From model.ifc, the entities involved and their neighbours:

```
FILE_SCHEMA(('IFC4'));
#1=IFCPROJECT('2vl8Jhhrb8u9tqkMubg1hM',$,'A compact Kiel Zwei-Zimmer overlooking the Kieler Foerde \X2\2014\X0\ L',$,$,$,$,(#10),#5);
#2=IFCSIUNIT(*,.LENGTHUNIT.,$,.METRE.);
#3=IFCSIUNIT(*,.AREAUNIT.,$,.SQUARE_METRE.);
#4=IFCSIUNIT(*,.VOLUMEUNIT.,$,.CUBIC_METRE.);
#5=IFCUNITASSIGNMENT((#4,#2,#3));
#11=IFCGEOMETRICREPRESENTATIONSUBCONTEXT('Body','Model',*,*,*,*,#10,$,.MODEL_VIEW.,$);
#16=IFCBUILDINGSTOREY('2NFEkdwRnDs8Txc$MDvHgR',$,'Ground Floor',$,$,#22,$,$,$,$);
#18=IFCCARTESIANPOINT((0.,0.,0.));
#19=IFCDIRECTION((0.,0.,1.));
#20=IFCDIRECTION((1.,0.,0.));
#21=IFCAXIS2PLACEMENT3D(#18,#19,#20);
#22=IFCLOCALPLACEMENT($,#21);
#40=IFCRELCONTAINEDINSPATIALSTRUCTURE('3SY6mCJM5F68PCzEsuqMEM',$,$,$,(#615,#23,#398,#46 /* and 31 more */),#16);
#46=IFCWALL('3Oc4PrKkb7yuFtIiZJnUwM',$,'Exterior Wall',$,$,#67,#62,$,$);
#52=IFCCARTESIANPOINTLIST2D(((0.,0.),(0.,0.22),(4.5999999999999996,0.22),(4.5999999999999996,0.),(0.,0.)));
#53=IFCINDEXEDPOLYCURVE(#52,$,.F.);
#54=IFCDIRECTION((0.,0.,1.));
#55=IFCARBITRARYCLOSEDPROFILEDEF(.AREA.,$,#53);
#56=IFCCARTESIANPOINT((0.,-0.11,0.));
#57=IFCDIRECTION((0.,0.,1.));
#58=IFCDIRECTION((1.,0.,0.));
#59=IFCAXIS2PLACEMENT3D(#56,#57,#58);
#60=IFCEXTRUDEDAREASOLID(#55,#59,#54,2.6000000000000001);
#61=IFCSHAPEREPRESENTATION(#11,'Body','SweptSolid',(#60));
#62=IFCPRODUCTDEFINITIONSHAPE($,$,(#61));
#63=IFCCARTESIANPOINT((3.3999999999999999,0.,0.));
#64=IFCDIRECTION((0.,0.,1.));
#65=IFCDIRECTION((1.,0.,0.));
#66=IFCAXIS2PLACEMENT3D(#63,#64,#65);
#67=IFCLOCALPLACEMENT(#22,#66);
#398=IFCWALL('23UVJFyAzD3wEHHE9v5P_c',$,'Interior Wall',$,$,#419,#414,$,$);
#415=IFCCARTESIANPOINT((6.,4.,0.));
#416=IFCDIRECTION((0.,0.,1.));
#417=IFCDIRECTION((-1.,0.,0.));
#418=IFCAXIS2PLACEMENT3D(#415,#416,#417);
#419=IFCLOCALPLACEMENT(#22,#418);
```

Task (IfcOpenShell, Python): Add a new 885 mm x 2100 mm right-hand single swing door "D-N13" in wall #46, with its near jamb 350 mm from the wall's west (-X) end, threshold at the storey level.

```python
import numpy as np
import ifcopenshell
import ifcopenshell.api.feature
import ifcopenshell.api.geometry
import ifcopenshell.api.root
import ifcopenshell.api.spatial
import ifcopenshell.geom
import ifcopenshell.util.element
import ifcopenshell.util.placement
import ifcopenshell.util.representation
import ifcopenshell.util.shape
import ifcopenshell.util.unit

model = ifcopenshell.open("model.ifc")
unit_scale = ifcopenshell.util.unit.calculate_unit_scale(model)
settings = ifcopenshell.geom.settings()


def volume(element):
    """Net volume in cubic metres, openings subtracted."""
    shape = ifcopenshell.geom.create_shape(settings, element)
    return ifcopenshell.util.shape.get_volume(shape.geometry)


wall = model.by_guid("3Oc4PrKkb7yuFtIiZJnUwM")
storey = ifcopenshell.util.element.get_container(wall, ifc_class="IfcBuildingStorey")
context = ifcopenshell.util.representation.get_context(model, "Model", "Body", "MODEL_VIEW")
before = volume(wall)

width, height, from_end, sill = 0.885, 2.1, 0.35, 0.0  # metres

# The wall runs along its own X axis, and the end named is its -X end.
wall_shape = ifcopenshell.geom.create_shape(settings, wall)
x, y, z = ifcopenshell.util.shape.get_vertices(wall_shape.geometry).T
start = x.min() + from_end
face, thickness = float(y.min()), float(y.max() - y.min())
wall_matrix = ifcopenshell.util.placement.get_local_placement(wall.ObjectPlacement)
level = ifcopenshell.util.placement.get_local_placement(storey.ObjectPlacement)[2, 3]


def in_wall(x, y):
    """Placement at x, y metres in the wall's axes, at sill height."""
    matrix = wall_matrix.copy()
    matrix[:, 3] = wall_matrix @ np.array([x / unit_scale, y / unit_scale, 0.0, 1.0])
    matrix[2, 3] = level + sill / unit_scale
    return matrix


# Opening: a box that overshoots both wall faces by 50 mm.
opening = ifcopenshell.api.root.create_entity(model, ifc_class="IfcOpeningElement", predefined_type="OPENING")
box = ifcopenshell.api.geometry.add_wall_representation(
    model, context=context, length=width, height=height, thickness=thickness + 0.1
)
ifcopenshell.api.geometry.assign_representation(model, product=opening, representation=box)
ifcopenshell.api.geometry.edit_object_placement(model, product=opening, matrix=in_wall(start, face - 0.05), is_si=False)
ifcopenshell.api.feature.add_feature(model, feature=opening, element=wall)

door = ifcopenshell.api.root.create_entity(model, ifc_class="IfcDoor", name="D-N13", predefined_type="DOOR")
door.OverallWidth, door.OverallHeight = width / unit_scale, height / unit_scale
door.OperationType = "SINGLE_SWING_RIGHT"
body = ifcopenshell.api.geometry.add_door_representation(
    model,
    context=context,
    overall_width=door.OverallWidth,
    overall_height=door.OverallHeight,
    operation_type="SINGLE_SWING_RIGHT",
    lining_properties={"LiningDepth": thickness / unit_scale, "ThresholdDepth": thickness / unit_scale},
)
ifcopenshell.api.geometry.assign_representation(model, product=door, representation=body)
ifcopenshell.api.spatial.assign_container(model, products=[door], relating_structure=storey)
ifcopenshell.api.feature.add_filling(model, opening=opening, element=door)

# The lining spans the wall, so the door starts at the wall face.
ifcopenshell.api.geometry.edit_object_placement(model, product=door, matrix=in_wall(start, face), is_si=False)

after = volume(wall)

print(f"wall volume {before:.3f} -> {after:.3f} m3")

model.write("model_edited.ifc")
```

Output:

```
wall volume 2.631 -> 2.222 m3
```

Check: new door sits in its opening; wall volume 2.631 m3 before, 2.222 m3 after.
